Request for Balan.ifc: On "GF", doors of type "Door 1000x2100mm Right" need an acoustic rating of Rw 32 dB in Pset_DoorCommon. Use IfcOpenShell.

First a look at what the model holds.

```python
import ifcopenshell
import ifcopenshell.util.element

model = ifcopenshell.open("Balan.ifc")
print(model.schema)
storey = next(s for s in model.by_type("IfcBuildingStorey") if s.Name == "GF")
doors = [e for e in ifcopenshell.util.element.get_decomposition(storey) if e.is_a("IfcDoor")]
seen = {}
for e in doors:
    element_type = ifcopenshell.util.element.get_type(e)
    key = (element_type.Name if element_type != e and element_type else None, ifcopenshell.util.element.get_pset(e, "Pset_DoorCommon", "AcousticRating"))
    seen[key] = seen.get(key, 0) + 1
for (name, value), count in sorted(seen.items(), key=str):
    print(count, "x", name, "|", value)
```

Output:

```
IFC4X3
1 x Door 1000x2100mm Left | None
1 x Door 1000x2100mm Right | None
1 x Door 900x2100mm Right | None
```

```python
import ifcopenshell
import ifcopenshell.api.pset
import ifcopenshell.util.element

model = ifcopenshell.open("Balan.ifc")

storey = next(s for s in model.by_type("IfcBuildingStorey") if s.Name == "GF")
doors = [e for e in ifcopenshell.util.element.get_decomposition(storey) if e.is_a("IfcDoor")]

count = 0
for e in doors:
    element_type = ifcopenshell.util.element.get_type(e)
    if element_type in (None, e) or element_type.Name != "Door 1000x2100mm Right":
        continue
    # add_pset returns the element's existing set when there is one.
    pset = ifcopenshell.api.pset.add_pset(model, product=e, name="Pset_DoorCommon")
    ifcopenshell.api.pset.edit_pset(model, pset=pset, properties={"AcousticRating": "Rw 32 dB"})
    count += 1

print(count, "doors updated")

model.write("Balan_edited.ifc")
```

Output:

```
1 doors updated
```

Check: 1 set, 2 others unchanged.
